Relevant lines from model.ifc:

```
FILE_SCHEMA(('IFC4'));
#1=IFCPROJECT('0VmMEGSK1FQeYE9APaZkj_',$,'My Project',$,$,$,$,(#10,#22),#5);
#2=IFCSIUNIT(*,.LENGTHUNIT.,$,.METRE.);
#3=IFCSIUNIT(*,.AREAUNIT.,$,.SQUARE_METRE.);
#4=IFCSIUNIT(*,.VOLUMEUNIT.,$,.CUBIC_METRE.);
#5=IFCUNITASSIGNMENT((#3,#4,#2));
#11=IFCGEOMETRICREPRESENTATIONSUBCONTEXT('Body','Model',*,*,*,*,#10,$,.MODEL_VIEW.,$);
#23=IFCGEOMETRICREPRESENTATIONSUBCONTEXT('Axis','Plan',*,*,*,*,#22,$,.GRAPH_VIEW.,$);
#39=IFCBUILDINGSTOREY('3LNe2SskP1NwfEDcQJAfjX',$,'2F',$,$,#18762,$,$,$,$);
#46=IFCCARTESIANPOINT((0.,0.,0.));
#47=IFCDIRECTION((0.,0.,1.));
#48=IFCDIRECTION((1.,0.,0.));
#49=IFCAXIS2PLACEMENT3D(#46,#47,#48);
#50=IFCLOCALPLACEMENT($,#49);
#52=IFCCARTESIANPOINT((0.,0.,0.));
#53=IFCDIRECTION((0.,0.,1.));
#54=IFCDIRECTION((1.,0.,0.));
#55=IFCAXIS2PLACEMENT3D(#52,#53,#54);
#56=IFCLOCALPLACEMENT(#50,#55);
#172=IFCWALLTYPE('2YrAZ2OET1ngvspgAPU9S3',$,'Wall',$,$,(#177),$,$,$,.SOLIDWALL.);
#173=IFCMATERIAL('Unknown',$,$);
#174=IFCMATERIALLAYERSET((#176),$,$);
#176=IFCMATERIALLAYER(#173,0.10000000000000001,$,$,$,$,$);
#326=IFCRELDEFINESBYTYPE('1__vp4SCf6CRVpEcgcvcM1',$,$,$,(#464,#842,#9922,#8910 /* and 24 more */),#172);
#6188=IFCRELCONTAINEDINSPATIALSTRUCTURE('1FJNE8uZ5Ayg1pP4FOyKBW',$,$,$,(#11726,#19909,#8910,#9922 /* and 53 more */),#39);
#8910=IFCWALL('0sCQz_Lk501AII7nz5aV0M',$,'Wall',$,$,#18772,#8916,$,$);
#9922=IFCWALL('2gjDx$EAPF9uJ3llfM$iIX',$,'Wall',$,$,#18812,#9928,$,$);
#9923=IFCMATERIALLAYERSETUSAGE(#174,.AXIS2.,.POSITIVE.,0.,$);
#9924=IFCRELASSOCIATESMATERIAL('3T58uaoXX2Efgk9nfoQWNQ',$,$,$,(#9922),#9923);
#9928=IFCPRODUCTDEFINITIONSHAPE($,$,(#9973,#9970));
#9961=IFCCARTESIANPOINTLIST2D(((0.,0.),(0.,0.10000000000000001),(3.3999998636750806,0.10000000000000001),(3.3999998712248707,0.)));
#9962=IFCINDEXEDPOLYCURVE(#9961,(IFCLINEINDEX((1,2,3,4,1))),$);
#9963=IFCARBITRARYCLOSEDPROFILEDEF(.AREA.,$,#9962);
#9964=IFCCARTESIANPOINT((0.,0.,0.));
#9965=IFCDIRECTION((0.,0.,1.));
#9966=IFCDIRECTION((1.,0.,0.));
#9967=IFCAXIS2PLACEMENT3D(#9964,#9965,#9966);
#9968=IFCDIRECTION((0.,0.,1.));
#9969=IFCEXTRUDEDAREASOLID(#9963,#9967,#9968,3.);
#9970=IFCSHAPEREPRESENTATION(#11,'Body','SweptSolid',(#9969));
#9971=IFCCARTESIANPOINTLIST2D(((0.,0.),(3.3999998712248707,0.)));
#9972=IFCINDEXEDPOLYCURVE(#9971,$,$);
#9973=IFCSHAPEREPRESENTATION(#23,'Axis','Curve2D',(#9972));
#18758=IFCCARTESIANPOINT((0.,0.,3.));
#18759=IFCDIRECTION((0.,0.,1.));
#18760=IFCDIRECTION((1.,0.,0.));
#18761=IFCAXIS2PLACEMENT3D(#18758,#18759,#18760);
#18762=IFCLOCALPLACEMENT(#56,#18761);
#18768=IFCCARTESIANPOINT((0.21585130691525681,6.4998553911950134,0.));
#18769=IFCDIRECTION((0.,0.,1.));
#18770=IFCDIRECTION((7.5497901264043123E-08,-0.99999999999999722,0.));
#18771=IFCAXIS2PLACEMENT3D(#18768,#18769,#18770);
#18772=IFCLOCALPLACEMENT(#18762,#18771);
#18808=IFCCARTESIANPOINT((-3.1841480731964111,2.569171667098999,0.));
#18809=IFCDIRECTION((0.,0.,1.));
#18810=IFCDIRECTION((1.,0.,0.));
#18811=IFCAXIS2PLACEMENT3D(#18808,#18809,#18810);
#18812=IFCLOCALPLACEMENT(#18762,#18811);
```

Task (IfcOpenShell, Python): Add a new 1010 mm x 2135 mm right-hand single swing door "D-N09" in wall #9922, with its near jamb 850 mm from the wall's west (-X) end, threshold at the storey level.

```python
import numpy as np
import ifcopenshell
import ifcopenshell.api.feature
import ifcopenshell.api.geometry
import ifcopenshell.api.root
import ifcopenshell.api.spatial
import ifcopenshell.geom
import ifcopenshell.util.element
import ifcopenshell.util.placement
import ifcopenshell.util.representation
import ifcopenshell.util.shape
import ifcopenshell.util.unit

model = ifcopenshell.open("model.ifc")
unit_scale = ifcopenshell.util.unit.calculate_unit_scale(model)
settings = ifcopenshell.geom.settings()


def volume(element):
    """Net volume in cubic metres, openings subtracted."""
    shape = ifcopenshell.geom.create_shape(settings, element)
    return ifcopenshell.util.shape.get_volume(shape.geometry)


wall = model.by_guid("2gjDx$EAPF9uJ3llfM$iIX")
storey = ifcopenshell.util.element.get_container(wall, ifc_class="IfcBuildingStorey")
context = ifcopenshell.util.representation.get_context(model, "Model", "Body", "MODEL_VIEW")
before = volume(wall)

width, height, from_end, sill = 1.01, 2.135, 0.85, 0.0  # metres

# The wall runs along its own X axis, and the end named is its -X end.
wall_shape = ifcopenshell.geom.create_shape(settings, wall)
x, y, z = ifcopenshell.util.shape.get_vertices(wall_shape.geometry).T
start = x.min() + from_end
face, thickness = float(y.min()), float(y.max() - y.min())
wall_matrix = ifcopenshell.util.placement.get_local_placement(wall.ObjectPlacement)
level = ifcopenshell.util.placement.get_local_placement(storey.ObjectPlacement)[2, 3]


def in_wall(x, y):
    """Placement at x, y metres in the wall's axes, at sill height."""
    matrix = wall_matrix.copy()
    matrix[:, 3] = wall_matrix @ np.array([x / unit_scale, y / unit_scale, 0.0, 1.0])
    matrix[2, 3] = level + sill / unit_scale
    return matrix


# Opening: a box that overshoots both wall faces by 50 mm.
opening = ifcopenshell.api.root.create_entity(model, ifc_class="IfcOpeningElement", predefined_type="OPENING")
box = ifcopenshell.api.geometry.add_wall_representation(
    model, context=context, length=width, height=height, thickness=thickness + 0.1
)
ifcopenshell.api.geometry.assign_representation(model, product=opening, representation=box)
ifcopenshell.api.geometry.edit_object_placement(model, product=opening, matrix=in_wall(start, face - 0.05), is_si=False)
ifcopenshell.api.feature.add_feature(model, feature=opening, element=wall)

door = ifcopenshell.api.root.create_entity(model, ifc_class="IfcDoor", name="D-N09", predefined_type="DOOR")
door.OverallWidth, door.OverallHeight = width / unit_scale, height / unit_scale
door.OperationType = "SINGLE_SWING_RIGHT"
body = ifcopenshell.api.geometry.add_door_representation(
    model,
    context=context,
    overall_width=door.OverallWidth,
    overall_height=door.OverallHeight,
    operation_type="SINGLE_SWING_RIGHT",
    lining_properties={"LiningDepth": thickness / unit_scale, "ThresholdDepth": thickness / unit_scale},
)
ifcopenshell.api.geometry.assign_representation(model, product=door, representation=body)
ifcopenshell.api.spatial.assign_container(model, products=[door], relating_structure=storey)
ifcopenshell.api.feature.add_filling(model, opening=opening, element=door)

# The lining spans the wall, so the door starts at the wall face.
ifcopenshell.api.geometry.edit_object_placement(model, product=door, matrix=in_wall(start, face), is_si=False)

after = volume(wall)

print(f"wall volume {before:.3f} -> {after:.3f} m3")

model.write("model-out.ifc")
```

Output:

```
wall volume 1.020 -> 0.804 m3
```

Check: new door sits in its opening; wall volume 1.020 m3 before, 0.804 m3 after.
